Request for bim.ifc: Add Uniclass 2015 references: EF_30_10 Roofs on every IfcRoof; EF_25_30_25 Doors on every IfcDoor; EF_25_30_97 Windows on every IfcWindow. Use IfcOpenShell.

First a look at what the model holds.

```python
import ifcopenshell

model = ifcopenshell.open("bim.ifc")
print(model.schema)
print("classifications:", [c.Name for c in model.by_type("IfcClassification")])
for ifc_class in ("IfcDoor", "IfcRoof", "IfcStair", "IfcWall", "IfcWindow"):
    print(ifc_class, len(model.by_type(ifc_class)))
```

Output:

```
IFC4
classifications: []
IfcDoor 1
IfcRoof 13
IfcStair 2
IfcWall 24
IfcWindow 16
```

```python
import ifcopenshell
import ifcopenshell.api.classification

model = ifcopenshell.open("bim.ifc")

system = ifcopenshell.api.classification.add_classification(model, classification="Uniclass 2015")

codes = {
    "IfcRoof": ("EF_30_10", "Roofs"),
    "IfcDoor": ("EF_25_30_25", "Doors"),
    "IfcWindow": ("EF_25_30_97", "Windows"),
}
for ifc_class, (code, name) in codes.items():
    products = model.by_type(ifc_class)
    ifcopenshell.api.classification.add_reference(
        model, products=products, classification=system, identification=code, name=name
    )
    print(code, len(products))

model.write("bim-out.ifc")
```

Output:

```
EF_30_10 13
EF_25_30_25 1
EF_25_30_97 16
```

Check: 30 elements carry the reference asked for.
